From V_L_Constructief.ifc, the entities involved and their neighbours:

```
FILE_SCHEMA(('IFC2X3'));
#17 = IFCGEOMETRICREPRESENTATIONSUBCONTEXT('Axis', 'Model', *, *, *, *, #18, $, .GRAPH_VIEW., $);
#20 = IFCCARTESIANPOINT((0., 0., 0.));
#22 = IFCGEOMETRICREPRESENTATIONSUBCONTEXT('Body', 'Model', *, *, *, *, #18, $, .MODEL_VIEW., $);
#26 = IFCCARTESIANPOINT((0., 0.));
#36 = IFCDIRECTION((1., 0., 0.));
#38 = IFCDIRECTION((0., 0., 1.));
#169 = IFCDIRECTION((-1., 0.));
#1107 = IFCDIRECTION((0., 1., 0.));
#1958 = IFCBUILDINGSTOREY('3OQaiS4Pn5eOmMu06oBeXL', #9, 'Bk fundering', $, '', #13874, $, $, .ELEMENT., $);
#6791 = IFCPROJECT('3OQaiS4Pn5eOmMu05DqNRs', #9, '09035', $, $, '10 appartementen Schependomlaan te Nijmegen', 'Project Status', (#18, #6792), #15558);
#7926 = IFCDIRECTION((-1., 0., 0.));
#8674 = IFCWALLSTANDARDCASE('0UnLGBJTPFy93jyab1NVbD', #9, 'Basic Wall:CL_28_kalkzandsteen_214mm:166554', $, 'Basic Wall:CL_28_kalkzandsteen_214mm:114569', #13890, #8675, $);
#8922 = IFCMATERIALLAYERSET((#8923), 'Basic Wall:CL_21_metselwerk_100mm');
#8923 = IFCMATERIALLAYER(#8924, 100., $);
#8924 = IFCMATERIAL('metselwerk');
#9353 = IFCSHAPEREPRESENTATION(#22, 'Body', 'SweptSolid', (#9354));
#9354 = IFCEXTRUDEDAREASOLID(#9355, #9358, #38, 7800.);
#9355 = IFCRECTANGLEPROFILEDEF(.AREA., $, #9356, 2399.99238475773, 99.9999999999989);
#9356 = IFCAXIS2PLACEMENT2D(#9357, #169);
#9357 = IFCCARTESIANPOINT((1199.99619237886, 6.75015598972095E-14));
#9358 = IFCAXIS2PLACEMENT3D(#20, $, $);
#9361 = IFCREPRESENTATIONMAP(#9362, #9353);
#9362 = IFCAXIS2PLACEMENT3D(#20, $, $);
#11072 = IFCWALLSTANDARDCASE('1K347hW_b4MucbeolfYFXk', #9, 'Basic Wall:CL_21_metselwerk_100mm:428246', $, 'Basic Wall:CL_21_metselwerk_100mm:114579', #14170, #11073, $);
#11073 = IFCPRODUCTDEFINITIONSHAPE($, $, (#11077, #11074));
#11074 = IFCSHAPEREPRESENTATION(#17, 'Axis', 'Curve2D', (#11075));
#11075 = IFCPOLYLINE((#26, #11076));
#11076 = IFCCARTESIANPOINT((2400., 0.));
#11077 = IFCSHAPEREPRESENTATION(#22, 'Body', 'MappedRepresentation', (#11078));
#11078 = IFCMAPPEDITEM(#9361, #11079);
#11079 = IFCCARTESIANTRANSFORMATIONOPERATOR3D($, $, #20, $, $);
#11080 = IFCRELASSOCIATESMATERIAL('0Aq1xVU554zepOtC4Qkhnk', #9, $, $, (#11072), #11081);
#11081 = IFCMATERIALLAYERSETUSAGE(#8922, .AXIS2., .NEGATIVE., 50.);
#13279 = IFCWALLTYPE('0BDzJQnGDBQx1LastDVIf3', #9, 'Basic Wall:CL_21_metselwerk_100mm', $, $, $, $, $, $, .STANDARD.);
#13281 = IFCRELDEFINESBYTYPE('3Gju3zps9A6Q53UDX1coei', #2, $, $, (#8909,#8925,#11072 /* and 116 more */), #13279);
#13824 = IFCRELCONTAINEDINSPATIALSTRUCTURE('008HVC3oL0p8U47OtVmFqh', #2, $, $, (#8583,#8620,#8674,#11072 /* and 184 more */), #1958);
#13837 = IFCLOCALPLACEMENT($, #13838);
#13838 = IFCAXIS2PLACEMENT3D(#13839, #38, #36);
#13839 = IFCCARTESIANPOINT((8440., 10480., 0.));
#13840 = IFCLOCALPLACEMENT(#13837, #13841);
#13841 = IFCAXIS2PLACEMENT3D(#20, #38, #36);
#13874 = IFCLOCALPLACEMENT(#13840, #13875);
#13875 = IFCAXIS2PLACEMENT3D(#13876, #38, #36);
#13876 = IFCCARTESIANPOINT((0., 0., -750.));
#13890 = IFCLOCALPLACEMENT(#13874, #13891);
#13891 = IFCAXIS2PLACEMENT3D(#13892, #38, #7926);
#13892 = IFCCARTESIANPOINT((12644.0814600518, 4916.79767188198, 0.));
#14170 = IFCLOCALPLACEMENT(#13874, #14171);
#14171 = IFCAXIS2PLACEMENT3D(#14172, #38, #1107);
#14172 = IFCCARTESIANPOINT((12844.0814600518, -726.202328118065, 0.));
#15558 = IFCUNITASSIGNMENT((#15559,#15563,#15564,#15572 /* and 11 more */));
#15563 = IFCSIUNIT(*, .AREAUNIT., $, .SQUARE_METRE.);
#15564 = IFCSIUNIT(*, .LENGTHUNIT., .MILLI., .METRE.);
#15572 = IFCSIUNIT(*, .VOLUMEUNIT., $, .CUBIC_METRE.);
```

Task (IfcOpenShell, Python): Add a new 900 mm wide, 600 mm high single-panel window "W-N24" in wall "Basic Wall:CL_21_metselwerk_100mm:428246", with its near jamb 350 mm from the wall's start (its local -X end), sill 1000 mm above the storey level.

```python
import numpy as np
import ifcopenshell
import ifcopenshell.api.feature
import ifcopenshell.api.geometry
import ifcopenshell.api.root
import ifcopenshell.api.spatial
import ifcopenshell.api.type
import ifcopenshell.geom
import ifcopenshell.util.element
import ifcopenshell.util.placement
import ifcopenshell.util.representation
import ifcopenshell.util.shape
import ifcopenshell.util.unit

model = ifcopenshell.open("V_L_Constructief.ifc")
unit_scale = ifcopenshell.util.unit.calculate_unit_scale(model)
settings = ifcopenshell.geom.settings()


def volume(element):
    """Net volume in cubic metres, openings subtracted."""
    shape = ifcopenshell.geom.create_shape(settings, element)
    return ifcopenshell.util.shape.get_volume(shape.geometry)


wall = model.by_guid("1K347hW_b4MucbeolfYFXk")
storey = ifcopenshell.util.element.get_container(wall, ifc_class="IfcBuildingStorey")
context = ifcopenshell.util.representation.get_context(model, "Model", "Body", "MODEL_VIEW")
before = volume(wall)

width, height, from_end, sill = 0.9, 0.6, 0.35, 1  # metres

# The wall runs along its own X axis, and the end named is its -X end.
wall_shape = ifcopenshell.geom.create_shape(settings, wall)
x, y, z = ifcopenshell.util.shape.get_vertices(wall_shape.geometry).T
start = x.min() + from_end
face, thickness = float(y.min()), float(y.max() - y.min())
wall_matrix = ifcopenshell.util.placement.get_local_placement(wall.ObjectPlacement)
level = ifcopenshell.util.placement.get_local_placement(storey.ObjectPlacement)[2, 3]


def in_wall(x, y):
    """Placement at x, y metres in the wall's axes, at sill height."""
    matrix = wall_matrix.copy()
    matrix[:, 3] = wall_matrix @ np.array([x / unit_scale, y / unit_scale, 0.0, 1.0])
    matrix[2, 3] = level + sill / unit_scale
    return matrix


# Opening: a box that overshoots both wall faces by 50 mm.
opening = ifcopenshell.api.root.create_entity(model, ifc_class="IfcOpeningElement")
box = ifcopenshell.api.geometry.add_wall_representation(
    model, context=context, length=width, height=height, thickness=thickness + 0.1
)
ifcopenshell.api.geometry.assign_representation(model, product=opening, representation=box)
ifcopenshell.api.geometry.edit_object_placement(model, product=opening, matrix=in_wall(start, face - 0.05), is_si=False)
ifcopenshell.api.feature.add_feature(model, feature=opening, element=wall)

window = ifcopenshell.api.root.create_entity(model, ifc_class="IfcWindow", name="W-N24")
window.OverallWidth, window.OverallHeight = width / unit_scale, height / unit_scale
body = ifcopenshell.api.geometry.add_window_representation(
    model,
    context=context,
    overall_width=window.OverallWidth,
    overall_height=window.OverallHeight,
    partition_type="SINGLE_PANEL",
)
ifcopenshell.api.geometry.assign_representation(model, product=window, representation=body)
ifcopenshell.api.spatial.assign_container(model, products=[window], relating_structure=storey)
fills = ifcopenshell.api.feature.add_filling(model, opening=opening, element=window)
fills.OwnerHistory = window.OwnerHistory  # required in IFC2X3

# IFC2X3 keeps the operation on the window style.
style = ifcopenshell.api.root.create_entity(model, ifc_class="IfcWindowStyle", name="W-N24")
style.OperationType, style.ConstructionType = "SINGLE_PANEL", "NOTDEFINED"
style.ParameterTakesPrecedence = style.Sizeable = False
ifcopenshell.api.type.assign_type(model, related_objects=[window], relating_type=style)

# Centre the window in the wall's thickness.
ifcopenshell.api.geometry.edit_object_placement(model, product=window, matrix=in_wall(start, face), is_si=False)
window_shape = ifcopenshell.geom.create_shape(settings, window)
depth = ifcopenshell.util.shape.get_vertices(window_shape.geometry)[:, 1]
offset = face + thickness / 2 - (depth.min() + depth.max()) / 2
ifcopenshell.api.geometry.edit_object_placement(model, product=window, matrix=in_wall(start, offset), is_si=False)

after = volume(wall)

print(f"wall volume {before:.3f} -> {after:.3f} m3")

model.write("V_L_Constructief_v2.ifc")
```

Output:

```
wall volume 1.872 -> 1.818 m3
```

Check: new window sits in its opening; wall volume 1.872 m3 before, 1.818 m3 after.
